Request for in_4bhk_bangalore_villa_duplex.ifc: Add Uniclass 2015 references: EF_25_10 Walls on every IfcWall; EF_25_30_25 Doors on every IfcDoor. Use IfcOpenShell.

First a look at what the model holds.

```python
import ifcopenshell

model = ifcopenshell.open("in_4bhk_bangalore_villa_duplex.ifc")
print(model.schema)
print("classifications:", [c.Name for c in model.by_type("IfcClassification")])
for ifc_class in ("IfcDoor", "IfcRoof", "IfcStair", "IfcWall", "IfcWindow"):
    print(ifc_class, len(model.by_type(ifc_class)))
```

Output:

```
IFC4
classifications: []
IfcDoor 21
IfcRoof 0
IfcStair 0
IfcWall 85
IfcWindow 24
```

```python
import ifcopenshell
import ifcopenshell.api.classification

model = ifcopenshell.open("in_4bhk_bangalore_villa_duplex.ifc")

system = ifcopenshell.api.classification.add_classification(model, classification="Uniclass 2015")

codes = {
    "IfcWall": ("EF_25_10", "Walls"),
    "IfcDoor": ("EF_25_30_25", "Doors"),
}
for ifc_class, (code, name) in codes.items():
    products = model.by_type(ifc_class)
    ifcopenshell.api.classification.add_reference(
        model, products=products, classification=system, identification=code, name=name
    )
    print(code, len(products))

model.write("in_4bhk_bangalore_villa_duplex-out.ifc")
```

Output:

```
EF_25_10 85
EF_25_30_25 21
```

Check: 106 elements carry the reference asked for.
